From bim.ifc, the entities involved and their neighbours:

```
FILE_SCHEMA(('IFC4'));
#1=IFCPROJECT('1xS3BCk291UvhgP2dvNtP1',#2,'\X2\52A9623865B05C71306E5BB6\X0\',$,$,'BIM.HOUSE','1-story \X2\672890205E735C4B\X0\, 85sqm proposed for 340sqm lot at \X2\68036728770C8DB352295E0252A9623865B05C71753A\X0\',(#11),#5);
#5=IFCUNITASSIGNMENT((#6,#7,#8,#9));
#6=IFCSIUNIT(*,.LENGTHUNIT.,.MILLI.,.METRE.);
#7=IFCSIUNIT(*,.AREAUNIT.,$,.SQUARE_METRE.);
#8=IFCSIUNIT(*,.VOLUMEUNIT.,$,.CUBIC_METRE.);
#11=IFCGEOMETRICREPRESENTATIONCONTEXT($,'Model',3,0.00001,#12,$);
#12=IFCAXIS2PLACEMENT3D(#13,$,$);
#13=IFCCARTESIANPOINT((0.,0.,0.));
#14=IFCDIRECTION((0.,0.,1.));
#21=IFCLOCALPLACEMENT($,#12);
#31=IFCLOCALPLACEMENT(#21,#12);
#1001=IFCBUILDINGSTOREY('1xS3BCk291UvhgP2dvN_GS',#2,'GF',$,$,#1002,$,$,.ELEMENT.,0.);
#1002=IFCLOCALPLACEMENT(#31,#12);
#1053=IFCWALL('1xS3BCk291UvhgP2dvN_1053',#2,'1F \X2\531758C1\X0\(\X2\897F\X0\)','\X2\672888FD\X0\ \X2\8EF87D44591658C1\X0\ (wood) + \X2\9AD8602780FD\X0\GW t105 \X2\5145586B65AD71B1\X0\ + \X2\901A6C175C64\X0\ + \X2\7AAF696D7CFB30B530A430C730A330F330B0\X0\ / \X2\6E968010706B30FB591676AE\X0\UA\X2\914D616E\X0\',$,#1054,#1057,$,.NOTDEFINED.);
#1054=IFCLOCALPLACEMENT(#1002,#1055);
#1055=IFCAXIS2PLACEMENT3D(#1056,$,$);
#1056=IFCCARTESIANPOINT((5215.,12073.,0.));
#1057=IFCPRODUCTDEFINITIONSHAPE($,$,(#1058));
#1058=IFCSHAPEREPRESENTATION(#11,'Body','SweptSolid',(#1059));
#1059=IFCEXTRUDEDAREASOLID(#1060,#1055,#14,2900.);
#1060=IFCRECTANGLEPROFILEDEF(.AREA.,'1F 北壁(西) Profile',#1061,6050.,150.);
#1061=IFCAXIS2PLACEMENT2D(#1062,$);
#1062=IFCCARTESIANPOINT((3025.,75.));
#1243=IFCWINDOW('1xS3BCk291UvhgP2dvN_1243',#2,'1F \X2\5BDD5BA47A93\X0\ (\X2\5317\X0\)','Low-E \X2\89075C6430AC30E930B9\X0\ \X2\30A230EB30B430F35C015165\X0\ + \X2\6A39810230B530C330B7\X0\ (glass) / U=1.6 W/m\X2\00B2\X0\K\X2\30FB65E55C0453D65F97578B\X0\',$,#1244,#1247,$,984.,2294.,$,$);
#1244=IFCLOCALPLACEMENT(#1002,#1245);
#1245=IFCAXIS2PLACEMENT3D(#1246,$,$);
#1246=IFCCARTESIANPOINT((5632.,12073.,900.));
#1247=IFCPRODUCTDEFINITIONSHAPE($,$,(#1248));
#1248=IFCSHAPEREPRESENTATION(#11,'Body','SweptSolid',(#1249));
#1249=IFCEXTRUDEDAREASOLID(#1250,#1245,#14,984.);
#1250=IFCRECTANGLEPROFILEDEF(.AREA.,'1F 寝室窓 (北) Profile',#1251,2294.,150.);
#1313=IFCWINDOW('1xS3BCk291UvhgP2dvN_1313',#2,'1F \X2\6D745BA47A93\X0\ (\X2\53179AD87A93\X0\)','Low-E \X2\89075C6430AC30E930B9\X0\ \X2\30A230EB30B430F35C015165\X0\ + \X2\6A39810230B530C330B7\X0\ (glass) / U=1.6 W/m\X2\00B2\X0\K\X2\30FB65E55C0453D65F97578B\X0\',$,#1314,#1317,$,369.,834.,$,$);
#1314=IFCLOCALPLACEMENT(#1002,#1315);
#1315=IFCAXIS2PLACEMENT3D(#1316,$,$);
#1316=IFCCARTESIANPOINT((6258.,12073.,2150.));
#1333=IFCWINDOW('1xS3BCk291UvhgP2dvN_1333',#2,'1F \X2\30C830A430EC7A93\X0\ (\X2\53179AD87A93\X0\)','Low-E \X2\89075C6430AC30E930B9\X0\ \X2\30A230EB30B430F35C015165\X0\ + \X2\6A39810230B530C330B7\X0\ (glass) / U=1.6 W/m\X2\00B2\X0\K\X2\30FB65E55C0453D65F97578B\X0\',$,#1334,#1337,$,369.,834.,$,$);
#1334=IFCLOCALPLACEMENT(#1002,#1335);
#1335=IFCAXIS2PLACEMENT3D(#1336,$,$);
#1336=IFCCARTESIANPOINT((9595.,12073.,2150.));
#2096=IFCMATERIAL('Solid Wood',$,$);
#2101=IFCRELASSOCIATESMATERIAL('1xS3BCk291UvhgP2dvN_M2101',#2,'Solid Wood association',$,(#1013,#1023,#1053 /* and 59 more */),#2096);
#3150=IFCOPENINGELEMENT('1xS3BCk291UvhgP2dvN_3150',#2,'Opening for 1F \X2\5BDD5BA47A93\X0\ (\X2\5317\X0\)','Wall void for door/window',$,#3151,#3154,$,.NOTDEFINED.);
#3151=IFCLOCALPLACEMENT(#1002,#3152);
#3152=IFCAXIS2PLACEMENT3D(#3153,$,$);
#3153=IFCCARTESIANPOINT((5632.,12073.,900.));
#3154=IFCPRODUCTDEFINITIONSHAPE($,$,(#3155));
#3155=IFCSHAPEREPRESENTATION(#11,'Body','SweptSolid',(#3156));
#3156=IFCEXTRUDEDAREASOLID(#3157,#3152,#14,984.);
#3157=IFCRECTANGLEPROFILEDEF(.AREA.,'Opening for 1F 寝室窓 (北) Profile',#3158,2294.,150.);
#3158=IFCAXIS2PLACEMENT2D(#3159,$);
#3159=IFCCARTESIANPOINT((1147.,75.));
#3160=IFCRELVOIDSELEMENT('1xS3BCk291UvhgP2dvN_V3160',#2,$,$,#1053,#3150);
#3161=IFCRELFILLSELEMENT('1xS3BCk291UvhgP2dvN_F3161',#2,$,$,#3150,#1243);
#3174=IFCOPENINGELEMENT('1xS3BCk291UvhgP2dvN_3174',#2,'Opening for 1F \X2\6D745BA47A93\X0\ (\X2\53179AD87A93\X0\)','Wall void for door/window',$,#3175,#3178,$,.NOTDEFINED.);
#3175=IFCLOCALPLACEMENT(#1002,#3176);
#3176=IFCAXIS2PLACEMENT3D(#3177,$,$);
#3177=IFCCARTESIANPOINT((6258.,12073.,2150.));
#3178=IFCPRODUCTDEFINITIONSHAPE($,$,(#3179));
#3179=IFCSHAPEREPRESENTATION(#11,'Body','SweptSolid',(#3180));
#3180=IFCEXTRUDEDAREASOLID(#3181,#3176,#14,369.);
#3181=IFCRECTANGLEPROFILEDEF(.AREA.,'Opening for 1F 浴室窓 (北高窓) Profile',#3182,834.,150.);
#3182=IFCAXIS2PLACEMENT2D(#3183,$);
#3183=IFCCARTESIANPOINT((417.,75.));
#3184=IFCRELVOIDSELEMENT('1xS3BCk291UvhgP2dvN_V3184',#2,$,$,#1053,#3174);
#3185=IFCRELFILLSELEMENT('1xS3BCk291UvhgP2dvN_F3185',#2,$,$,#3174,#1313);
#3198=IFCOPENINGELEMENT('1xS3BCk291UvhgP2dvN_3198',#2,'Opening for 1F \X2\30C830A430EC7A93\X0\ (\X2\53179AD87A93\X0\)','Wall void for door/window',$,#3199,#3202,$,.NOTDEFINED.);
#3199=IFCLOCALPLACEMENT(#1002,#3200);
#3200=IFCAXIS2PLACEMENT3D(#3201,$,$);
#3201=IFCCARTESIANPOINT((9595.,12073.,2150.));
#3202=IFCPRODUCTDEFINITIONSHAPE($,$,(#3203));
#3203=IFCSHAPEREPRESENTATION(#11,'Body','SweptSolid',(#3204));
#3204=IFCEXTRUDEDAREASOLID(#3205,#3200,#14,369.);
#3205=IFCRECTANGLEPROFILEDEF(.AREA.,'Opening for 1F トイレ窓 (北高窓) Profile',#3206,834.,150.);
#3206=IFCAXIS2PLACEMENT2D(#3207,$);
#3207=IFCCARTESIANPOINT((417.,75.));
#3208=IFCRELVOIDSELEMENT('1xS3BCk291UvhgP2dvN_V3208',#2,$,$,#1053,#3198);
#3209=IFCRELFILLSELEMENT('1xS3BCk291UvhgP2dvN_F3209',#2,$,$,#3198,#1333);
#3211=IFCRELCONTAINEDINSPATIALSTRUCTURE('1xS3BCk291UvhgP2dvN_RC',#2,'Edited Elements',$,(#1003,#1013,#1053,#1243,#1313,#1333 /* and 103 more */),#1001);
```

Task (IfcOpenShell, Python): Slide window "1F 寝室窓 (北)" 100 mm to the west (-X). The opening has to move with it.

```python
import ifcopenshell
import ifcopenshell.api.geometry
import ifcopenshell.util.placement

model = ifcopenshell.open("bim.ifc")

window = model.by_id(1243)
opening = window.FillsVoids[0].RelatingOpeningElement
wall = opening.VoidsElements[0].RelatingBuildingElement

wall_matrix = ifcopenshell.util.placement.get_local_placement(wall.ObjectPlacement)
shift = wall_matrix[:3, 0] * -100.0
before = ifcopenshell.util.placement.get_local_placement(window.ObjectPlacement)[:3, 3].copy()

# The window is not placed relative to its opening, so move both.
for product in (opening, window):
    matrix = ifcopenshell.util.placement.get_local_placement(product.ObjectPlacement)
    matrix[:3, 3] += shift
    ifcopenshell.api.geometry.edit_object_placement(model, product=product, matrix=matrix, is_si=False)

after = ifcopenshell.util.placement.get_local_placement(window.ObjectPlacement)[:3, 3]
print("window moved by", (after - before).round(3) + 0.0)

model.write("bim_rev.ifc")
```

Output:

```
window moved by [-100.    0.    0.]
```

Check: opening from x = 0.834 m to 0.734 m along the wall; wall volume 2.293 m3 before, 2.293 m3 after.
